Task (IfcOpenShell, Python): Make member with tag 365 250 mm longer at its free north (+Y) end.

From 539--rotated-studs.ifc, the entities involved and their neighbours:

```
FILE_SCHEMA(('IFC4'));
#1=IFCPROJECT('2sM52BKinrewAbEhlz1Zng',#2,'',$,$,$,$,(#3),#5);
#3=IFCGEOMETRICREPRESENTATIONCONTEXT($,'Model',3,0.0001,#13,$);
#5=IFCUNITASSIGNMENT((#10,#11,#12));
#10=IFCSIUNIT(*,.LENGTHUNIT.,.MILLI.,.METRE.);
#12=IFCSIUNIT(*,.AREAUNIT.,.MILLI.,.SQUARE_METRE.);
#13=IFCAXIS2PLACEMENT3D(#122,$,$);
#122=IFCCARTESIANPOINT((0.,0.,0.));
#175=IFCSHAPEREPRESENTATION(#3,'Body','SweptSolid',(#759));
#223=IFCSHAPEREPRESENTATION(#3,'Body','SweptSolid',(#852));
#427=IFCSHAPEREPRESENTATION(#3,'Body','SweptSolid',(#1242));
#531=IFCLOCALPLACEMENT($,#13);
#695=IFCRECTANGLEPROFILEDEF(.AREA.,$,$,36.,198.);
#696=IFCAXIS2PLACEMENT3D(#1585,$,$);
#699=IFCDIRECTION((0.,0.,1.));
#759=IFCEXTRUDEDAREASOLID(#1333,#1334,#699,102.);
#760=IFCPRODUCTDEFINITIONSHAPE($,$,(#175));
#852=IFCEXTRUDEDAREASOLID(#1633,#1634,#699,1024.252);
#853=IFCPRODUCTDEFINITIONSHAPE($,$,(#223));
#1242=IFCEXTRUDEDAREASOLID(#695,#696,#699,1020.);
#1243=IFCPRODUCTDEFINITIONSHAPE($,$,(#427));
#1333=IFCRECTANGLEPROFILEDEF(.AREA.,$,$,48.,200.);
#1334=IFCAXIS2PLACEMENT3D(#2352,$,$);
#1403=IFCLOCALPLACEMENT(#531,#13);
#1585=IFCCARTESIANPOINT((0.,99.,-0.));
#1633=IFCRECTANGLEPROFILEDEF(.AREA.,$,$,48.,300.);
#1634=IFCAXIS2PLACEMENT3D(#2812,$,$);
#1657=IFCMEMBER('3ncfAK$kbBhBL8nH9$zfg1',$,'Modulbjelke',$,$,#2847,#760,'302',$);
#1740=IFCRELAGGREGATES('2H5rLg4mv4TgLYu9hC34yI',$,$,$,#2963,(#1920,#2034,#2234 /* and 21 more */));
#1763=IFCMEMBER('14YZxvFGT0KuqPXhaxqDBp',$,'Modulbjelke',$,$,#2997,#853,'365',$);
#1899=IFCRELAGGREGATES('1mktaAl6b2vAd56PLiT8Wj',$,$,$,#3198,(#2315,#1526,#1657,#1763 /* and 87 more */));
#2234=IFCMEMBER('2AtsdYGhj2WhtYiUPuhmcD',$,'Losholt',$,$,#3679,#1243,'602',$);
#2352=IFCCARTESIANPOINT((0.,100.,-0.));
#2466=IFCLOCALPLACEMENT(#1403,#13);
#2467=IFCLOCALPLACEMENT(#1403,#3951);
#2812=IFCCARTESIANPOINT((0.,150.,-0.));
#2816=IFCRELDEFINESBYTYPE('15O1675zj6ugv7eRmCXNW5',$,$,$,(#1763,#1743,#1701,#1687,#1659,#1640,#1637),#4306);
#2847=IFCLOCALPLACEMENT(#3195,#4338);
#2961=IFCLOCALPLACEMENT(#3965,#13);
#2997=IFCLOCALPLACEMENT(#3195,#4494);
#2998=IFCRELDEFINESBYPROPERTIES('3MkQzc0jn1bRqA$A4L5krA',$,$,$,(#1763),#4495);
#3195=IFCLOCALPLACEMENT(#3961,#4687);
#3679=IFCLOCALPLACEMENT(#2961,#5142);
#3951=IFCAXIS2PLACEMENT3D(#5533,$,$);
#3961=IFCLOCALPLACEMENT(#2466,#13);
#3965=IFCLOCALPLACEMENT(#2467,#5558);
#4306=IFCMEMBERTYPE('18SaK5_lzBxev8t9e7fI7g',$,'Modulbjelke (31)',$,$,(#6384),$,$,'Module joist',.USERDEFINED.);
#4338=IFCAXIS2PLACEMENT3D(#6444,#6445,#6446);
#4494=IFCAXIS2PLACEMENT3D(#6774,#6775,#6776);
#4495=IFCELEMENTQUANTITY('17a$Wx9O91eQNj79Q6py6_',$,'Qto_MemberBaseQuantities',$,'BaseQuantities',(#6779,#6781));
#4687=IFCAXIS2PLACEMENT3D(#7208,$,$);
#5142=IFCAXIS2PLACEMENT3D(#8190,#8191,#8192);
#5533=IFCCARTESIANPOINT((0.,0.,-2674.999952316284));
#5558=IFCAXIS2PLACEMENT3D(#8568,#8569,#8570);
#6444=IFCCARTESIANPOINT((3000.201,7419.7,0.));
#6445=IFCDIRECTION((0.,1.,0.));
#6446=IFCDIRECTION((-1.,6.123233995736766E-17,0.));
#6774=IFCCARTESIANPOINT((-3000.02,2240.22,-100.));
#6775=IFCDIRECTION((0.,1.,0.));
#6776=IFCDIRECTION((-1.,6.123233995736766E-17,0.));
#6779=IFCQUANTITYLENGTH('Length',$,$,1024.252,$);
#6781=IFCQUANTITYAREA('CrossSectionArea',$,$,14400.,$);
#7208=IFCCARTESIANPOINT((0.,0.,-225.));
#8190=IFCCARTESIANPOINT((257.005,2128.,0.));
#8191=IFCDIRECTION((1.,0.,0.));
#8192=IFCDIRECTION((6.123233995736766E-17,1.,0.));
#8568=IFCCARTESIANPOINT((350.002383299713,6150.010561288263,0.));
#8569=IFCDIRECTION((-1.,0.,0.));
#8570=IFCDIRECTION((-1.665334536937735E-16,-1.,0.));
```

```python
import ifcopenshell
import ifcopenshell.api.pset
import ifcopenshell.util.element
import ifcopenshell.util.unit

model = ifcopenshell.open("539--rotated-studs.ifc")
unit_scale = ifcopenshell.util.unit.calculate_unit_scale(model)

member = model.by_guid("14YZxvFGT0KuqPXhaxqDBp")
change = 0.25 / unit_scale

# The extrusion runs towards the end named, so only its depth changes.
body = next(r for r in member.Representation.Representations if r.RepresentationIdentifier == "Body")
solid = body.Items[0]
old_length = solid.Depth
solid.Depth += change

# Update the stored length and volume.
qto = model.by_id(ifcopenshell.util.element.get_pset(member, "Qto_MemberBaseQuantities", should_inherit=False)["id"])
ifcopenshell.api.pset.edit_qto(model, qto=qto, properties={"Length": solid.Depth})

print(f"length {old_length:g} -> {solid.Depth:g}")

model.write("539--rotated-studs_v2.ifc")
```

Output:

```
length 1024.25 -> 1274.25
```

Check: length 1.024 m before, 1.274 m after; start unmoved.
